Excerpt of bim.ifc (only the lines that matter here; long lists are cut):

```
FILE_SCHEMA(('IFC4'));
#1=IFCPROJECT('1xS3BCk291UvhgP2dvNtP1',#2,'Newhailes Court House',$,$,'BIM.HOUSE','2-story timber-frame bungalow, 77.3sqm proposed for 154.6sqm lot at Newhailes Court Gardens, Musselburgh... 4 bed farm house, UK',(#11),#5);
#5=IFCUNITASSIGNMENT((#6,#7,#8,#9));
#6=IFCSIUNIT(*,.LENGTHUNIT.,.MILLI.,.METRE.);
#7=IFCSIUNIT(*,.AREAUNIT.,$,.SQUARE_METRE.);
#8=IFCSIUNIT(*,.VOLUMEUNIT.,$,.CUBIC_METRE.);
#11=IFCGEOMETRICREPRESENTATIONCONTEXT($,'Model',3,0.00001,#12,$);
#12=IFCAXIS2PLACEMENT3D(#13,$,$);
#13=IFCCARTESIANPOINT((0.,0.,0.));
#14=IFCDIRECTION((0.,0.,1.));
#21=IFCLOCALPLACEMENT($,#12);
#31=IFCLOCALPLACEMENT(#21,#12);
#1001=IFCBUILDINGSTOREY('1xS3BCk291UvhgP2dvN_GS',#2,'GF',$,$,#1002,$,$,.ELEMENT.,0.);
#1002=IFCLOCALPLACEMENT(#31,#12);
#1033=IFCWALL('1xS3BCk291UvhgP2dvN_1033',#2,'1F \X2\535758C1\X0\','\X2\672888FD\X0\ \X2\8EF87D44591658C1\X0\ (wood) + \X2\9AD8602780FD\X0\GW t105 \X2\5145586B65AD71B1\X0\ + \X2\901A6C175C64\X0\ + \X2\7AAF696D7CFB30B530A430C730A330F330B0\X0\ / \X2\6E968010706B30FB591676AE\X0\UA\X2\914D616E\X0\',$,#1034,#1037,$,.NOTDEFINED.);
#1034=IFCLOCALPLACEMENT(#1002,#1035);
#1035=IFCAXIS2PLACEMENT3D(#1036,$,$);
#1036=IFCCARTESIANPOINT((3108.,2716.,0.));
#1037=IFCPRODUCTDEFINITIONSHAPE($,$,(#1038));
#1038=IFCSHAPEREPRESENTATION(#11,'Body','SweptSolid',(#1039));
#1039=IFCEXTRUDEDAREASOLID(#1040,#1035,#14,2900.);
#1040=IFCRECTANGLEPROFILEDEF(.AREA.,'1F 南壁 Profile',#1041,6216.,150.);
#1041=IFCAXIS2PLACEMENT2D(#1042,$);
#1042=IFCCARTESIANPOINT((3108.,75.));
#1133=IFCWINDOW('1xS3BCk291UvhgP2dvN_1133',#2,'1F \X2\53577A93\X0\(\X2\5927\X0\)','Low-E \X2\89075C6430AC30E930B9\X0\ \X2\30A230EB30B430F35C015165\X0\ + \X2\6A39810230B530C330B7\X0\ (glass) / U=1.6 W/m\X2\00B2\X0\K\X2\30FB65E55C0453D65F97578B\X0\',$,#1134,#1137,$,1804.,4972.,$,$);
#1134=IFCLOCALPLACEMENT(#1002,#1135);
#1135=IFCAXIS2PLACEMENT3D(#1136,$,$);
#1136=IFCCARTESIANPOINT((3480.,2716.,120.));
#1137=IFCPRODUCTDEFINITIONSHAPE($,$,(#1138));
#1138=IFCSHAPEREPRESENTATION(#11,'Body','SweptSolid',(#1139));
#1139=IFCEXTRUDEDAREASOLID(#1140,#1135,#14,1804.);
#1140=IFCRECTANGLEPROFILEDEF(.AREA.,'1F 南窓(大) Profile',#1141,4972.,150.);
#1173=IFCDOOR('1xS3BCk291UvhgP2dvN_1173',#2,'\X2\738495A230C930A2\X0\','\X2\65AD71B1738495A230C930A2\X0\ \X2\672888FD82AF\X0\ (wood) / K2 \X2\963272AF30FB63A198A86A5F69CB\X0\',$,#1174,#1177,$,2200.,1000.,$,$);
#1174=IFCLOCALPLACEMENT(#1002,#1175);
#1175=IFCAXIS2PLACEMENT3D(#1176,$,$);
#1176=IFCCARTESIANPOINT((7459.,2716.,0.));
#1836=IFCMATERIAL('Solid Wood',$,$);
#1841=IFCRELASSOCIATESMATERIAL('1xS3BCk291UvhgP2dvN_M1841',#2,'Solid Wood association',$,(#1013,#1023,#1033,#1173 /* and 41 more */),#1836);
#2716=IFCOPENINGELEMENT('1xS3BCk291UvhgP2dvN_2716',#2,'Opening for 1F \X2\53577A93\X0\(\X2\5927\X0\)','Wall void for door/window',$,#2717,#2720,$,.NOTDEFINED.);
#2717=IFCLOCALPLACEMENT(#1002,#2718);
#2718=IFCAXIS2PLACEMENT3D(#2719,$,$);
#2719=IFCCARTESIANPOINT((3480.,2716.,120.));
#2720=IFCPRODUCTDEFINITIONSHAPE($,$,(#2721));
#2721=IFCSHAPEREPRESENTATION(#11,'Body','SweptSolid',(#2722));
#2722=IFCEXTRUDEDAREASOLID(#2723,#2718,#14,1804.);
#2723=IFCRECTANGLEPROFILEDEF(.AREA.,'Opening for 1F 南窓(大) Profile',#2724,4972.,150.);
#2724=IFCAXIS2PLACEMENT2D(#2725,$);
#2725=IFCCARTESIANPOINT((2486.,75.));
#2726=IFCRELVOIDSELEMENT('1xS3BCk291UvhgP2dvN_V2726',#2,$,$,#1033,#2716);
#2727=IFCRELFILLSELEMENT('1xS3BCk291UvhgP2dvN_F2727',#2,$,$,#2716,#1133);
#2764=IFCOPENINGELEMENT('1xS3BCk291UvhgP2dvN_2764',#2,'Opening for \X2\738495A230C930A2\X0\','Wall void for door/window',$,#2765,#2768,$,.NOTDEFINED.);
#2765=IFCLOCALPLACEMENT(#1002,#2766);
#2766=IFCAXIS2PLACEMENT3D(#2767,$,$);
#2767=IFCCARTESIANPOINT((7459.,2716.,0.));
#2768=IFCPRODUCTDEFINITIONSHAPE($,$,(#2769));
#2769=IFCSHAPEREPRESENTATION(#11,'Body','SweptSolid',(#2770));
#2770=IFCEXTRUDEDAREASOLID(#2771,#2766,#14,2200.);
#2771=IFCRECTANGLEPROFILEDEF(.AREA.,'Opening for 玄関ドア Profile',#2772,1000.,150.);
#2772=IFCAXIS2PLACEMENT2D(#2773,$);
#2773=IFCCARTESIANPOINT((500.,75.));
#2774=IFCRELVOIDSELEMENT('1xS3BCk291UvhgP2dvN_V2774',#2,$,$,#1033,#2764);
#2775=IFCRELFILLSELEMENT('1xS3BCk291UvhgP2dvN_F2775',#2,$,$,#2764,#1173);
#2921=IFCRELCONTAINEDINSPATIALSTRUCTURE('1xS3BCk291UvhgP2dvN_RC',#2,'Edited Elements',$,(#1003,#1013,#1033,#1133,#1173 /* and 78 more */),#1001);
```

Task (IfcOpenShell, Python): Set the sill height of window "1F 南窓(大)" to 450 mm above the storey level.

```python
import numpy as np
import ifcopenshell
import ifcopenshell.api.geometry
import ifcopenshell.geom
import ifcopenshell.util.element
import ifcopenshell.util.placement
import ifcopenshell.util.shape
import ifcopenshell.util.unit

model = ifcopenshell.open("bim.ifc")
unit_scale = ifcopenshell.util.unit.calculate_unit_scale(model)

window = model.by_id(1133)
opening = window.FillsVoids[0].RelatingOpeningElement
storey = ifcopenshell.util.element.get_container(window, ifc_class="IfcBuildingStorey")
level = ifcopenshell.util.placement.get_local_placement(storey.ObjectPlacement)[2, 3]

# The opening's origin need not be at the sill, so measure its lowest point.
shape = ifcopenshell.geom.create_shape(ifcopenshell.geom.settings(), opening)
bottom = ifcopenshell.util.shape.get_shape_bottom_elevation(shape, shape.geometry) / unit_scale
dz = level + 0.45 / unit_scale - bottom

shift = np.array([0.0, 0.0, dz])
# The window is not placed relative to its opening, so move both.
for product in (opening, window):
    matrix = ifcopenshell.util.placement.get_local_placement(product.ObjectPlacement)
    matrix[:3, 3] += shift
    ifcopenshell.api.geometry.edit_object_placement(model, product=product, matrix=matrix, is_si=False)

print(f"moved by {dz * unit_scale:+.3f} m")

model.write("bim_v2.ifc")
```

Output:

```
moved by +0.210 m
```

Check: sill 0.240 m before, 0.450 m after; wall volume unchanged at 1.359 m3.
